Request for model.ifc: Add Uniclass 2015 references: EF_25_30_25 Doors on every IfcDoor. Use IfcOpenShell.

First a look at what the model holds.

```python
import ifcopenshell

model = ifcopenshell.open("model.ifc")
print(model.schema)
print("classifications:", [c.Name for c in model.by_type("IfcClassification")])
for ifc_class in ("IfcDoor", "IfcRoof", "IfcStair", "IfcWall", "IfcWindow"):
    print(ifc_class, len(model.by_type(ifc_class)))
```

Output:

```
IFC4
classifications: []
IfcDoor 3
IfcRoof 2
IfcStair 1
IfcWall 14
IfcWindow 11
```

```python
import ifcopenshell
import ifcopenshell.api.classification

model = ifcopenshell.open("model.ifc")

system = ifcopenshell.api.classification.add_classification(model, classification="Uniclass 2015")

codes = {
    "IfcDoor": ("EF_25_30_25", "Doors"),
}
for ifc_class, (code, name) in codes.items():
    products = model.by_type(ifc_class)
    ifcopenshell.api.classification.add_reference(
        model, products=products, classification=system, identification=code, name=name
    )
    print(code, len(products))

model.write("model-out.ifc")
```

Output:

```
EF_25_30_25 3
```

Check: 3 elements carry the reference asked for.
